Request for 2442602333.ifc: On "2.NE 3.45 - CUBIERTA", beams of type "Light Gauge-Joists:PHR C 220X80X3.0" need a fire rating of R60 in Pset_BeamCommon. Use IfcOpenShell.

First a look at what the model holds.

```python
import ifcopenshell
import ifcopenshell.util.element

model = ifcopenshell.open("2442602333.ifc")
print(model.schema)
storey = next(s for s in model.by_type("IfcBuildingStorey") if s.Name == "2.NE 3.45 - CUBIERTA")
beams = [e for e in ifcopenshell.util.element.get_decomposition(storey) if e.is_a("IfcBeam")]
seen = {}
for e in beams:
    element_type = ifcopenshell.util.element.get_type(e)
    key = (element_type.Name if element_type != e and element_type else None, ifcopenshell.util.element.get_pset(e, "Pset_BeamCommon", "FireRating"))
    seen[key] = seen.get(key, 0) + 1
for (name, value), count in sorted(seen.items(), key=str):
    print(count, "x", name, "|", value)
```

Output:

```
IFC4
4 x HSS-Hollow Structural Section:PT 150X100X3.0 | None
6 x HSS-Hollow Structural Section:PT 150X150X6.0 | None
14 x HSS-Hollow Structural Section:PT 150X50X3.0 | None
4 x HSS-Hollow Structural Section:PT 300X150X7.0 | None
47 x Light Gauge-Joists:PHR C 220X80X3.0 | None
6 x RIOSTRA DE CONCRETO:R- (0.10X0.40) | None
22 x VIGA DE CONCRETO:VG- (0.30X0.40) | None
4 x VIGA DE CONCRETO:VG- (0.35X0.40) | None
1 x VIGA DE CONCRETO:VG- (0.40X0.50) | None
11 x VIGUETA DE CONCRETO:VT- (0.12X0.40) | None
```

```python
import ifcopenshell
import ifcopenshell.api.pset
import ifcopenshell.util.element

model = ifcopenshell.open("2442602333.ifc")

storey = next(s for s in model.by_type("IfcBuildingStorey") if s.Name == "2.NE 3.45 - CUBIERTA")
beams = [e for e in ifcopenshell.util.element.get_decomposition(storey) if e.is_a("IfcBeam")]

count = 0
for e in beams:
    element_type = ifcopenshell.util.element.get_type(e)
    if element_type in (None, e) or element_type.Name != "Light Gauge-Joists:PHR C 220X80X3.0":
        continue
    # add_pset returns the element's existing set when there is one.
    pset = ifcopenshell.api.pset.add_pset(model, product=e, name="Pset_BeamCommon")
    ifcopenshell.api.pset.edit_pset(model, pset=pset, properties={"FireRating": "R60"})
    count += 1

print(count, "beams updated")

model.write("2442602333_edited.ifc")
```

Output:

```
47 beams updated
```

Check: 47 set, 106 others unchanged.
